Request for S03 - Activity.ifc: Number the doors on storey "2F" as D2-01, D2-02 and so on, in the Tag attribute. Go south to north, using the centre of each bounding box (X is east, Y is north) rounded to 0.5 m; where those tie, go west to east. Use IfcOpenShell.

First a look at what the model holds.

```python
import ifcopenshell
import ifcopenshell.util.element
import ifcopenshell.util.placement

model = ifcopenshell.open("S03 - Activity.ifc")
print(model.schema)
storey = next(s for s in model.by_type("IfcBuildingStorey") if s.Name == "2F")
doors = [e for e in ifcopenshell.util.element.get_decomposition(storey) if e.is_a("IfcDoor")]
for e in sorted(doors, key=lambda e: e.id()):
    origin = ifcopenshell.util.placement.get_local_placement(e.ObjectPlacement)[:3, 3]
    print(e.id(), e.Tag, e.Name, origin.round(2) + 0.0, sep=" | ")
```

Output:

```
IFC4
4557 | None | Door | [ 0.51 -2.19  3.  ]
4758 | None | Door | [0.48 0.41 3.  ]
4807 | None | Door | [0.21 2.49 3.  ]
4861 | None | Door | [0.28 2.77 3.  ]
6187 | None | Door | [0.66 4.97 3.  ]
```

```python
import ifcopenshell
import ifcopenshell.geom
import ifcopenshell.util.element
import ifcopenshell.util.shape

model = ifcopenshell.open("S03 - Activity.ifc")
settings = ifcopenshell.geom.settings()
settings.set("use-world-coords", True)


def centre(element):
    shape = ifcopenshell.geom.create_shape(settings, element)
    return ifcopenshell.util.shape.get_bbox_centroid(shape.geometry)


storey = next(s for s in model.by_type("IfcBuildingStorey") if s.Name == "2F")
doors = [e for e in ifcopenshell.util.element.get_decomposition(storey) if e.is_a("IfcDoor")]

# Insertion points can sit at a corner or the storey origin, so sort by the geometry (in metres).
centres = {e: centre(e) for e in doors}
doors.sort(key=lambda e: (round(centres[e][1] / 0.5), centres[e][0]))

for i, e in enumerate(doors, start=1):
    number = f"D2-{i:02d}"
    e.Tag = number
    print(e.id(), number)

model.write("S03 - Activity_v2.ifc")
```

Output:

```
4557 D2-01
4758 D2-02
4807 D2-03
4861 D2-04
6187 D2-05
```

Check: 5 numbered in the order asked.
